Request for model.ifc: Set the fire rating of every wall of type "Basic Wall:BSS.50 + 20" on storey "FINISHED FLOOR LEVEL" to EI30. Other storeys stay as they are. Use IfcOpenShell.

First a look at what the model holds.

```python
import ifcopenshell
import ifcopenshell.util.element

model = ifcopenshell.open("model.ifc")
print(model.schema)
storey = next(s for s in model.by_type("IfcBuildingStorey") if s.Name == "FINISHED FLOOR LEVEL")
walls = [e for e in ifcopenshell.util.element.get_decomposition(storey) if e.is_a("IfcWall")]
seen = {}
for e in walls:
    element_type = ifcopenshell.util.element.get_type(e)
    key = (element_type.Name if element_type != e and element_type else None, ifcopenshell.util.element.get_pset(e, "Pset_WallCommon", "FireRating"))
    seen[key] = seen.get(key, 0) + 1
for (name, value), count in sorted(seen.items(), key=str):
    print(count, "x", name, "|", value)
```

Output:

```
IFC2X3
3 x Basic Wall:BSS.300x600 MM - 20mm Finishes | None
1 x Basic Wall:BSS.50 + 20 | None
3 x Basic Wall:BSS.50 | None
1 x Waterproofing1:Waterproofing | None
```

```python
import ifcopenshell
import ifcopenshell.api.pset
import ifcopenshell.util.element

model = ifcopenshell.open("model.ifc")

storey = next(s for s in model.by_type("IfcBuildingStorey") if s.Name == "FINISHED FLOOR LEVEL")
walls = [e for e in ifcopenshell.util.element.get_decomposition(storey) if e.is_a("IfcWall")]

count = 0
for e in walls:
    element_type = ifcopenshell.util.element.get_type(e)
    if element_type in (None, e) or element_type.Name != "Basic Wall:BSS.50 + 20":
        continue
    # add_pset returns the element's existing set when there is one.
    pset = ifcopenshell.api.pset.add_pset(model, product=e, name="Pset_WallCommon")
    ifcopenshell.api.pset.edit_pset(model, pset=pset, properties={"FireRating": "EI30"})
    count += 1

print(count, "walls updated")

model.write("model_rev.ifc")
```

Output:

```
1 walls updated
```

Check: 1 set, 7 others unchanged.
